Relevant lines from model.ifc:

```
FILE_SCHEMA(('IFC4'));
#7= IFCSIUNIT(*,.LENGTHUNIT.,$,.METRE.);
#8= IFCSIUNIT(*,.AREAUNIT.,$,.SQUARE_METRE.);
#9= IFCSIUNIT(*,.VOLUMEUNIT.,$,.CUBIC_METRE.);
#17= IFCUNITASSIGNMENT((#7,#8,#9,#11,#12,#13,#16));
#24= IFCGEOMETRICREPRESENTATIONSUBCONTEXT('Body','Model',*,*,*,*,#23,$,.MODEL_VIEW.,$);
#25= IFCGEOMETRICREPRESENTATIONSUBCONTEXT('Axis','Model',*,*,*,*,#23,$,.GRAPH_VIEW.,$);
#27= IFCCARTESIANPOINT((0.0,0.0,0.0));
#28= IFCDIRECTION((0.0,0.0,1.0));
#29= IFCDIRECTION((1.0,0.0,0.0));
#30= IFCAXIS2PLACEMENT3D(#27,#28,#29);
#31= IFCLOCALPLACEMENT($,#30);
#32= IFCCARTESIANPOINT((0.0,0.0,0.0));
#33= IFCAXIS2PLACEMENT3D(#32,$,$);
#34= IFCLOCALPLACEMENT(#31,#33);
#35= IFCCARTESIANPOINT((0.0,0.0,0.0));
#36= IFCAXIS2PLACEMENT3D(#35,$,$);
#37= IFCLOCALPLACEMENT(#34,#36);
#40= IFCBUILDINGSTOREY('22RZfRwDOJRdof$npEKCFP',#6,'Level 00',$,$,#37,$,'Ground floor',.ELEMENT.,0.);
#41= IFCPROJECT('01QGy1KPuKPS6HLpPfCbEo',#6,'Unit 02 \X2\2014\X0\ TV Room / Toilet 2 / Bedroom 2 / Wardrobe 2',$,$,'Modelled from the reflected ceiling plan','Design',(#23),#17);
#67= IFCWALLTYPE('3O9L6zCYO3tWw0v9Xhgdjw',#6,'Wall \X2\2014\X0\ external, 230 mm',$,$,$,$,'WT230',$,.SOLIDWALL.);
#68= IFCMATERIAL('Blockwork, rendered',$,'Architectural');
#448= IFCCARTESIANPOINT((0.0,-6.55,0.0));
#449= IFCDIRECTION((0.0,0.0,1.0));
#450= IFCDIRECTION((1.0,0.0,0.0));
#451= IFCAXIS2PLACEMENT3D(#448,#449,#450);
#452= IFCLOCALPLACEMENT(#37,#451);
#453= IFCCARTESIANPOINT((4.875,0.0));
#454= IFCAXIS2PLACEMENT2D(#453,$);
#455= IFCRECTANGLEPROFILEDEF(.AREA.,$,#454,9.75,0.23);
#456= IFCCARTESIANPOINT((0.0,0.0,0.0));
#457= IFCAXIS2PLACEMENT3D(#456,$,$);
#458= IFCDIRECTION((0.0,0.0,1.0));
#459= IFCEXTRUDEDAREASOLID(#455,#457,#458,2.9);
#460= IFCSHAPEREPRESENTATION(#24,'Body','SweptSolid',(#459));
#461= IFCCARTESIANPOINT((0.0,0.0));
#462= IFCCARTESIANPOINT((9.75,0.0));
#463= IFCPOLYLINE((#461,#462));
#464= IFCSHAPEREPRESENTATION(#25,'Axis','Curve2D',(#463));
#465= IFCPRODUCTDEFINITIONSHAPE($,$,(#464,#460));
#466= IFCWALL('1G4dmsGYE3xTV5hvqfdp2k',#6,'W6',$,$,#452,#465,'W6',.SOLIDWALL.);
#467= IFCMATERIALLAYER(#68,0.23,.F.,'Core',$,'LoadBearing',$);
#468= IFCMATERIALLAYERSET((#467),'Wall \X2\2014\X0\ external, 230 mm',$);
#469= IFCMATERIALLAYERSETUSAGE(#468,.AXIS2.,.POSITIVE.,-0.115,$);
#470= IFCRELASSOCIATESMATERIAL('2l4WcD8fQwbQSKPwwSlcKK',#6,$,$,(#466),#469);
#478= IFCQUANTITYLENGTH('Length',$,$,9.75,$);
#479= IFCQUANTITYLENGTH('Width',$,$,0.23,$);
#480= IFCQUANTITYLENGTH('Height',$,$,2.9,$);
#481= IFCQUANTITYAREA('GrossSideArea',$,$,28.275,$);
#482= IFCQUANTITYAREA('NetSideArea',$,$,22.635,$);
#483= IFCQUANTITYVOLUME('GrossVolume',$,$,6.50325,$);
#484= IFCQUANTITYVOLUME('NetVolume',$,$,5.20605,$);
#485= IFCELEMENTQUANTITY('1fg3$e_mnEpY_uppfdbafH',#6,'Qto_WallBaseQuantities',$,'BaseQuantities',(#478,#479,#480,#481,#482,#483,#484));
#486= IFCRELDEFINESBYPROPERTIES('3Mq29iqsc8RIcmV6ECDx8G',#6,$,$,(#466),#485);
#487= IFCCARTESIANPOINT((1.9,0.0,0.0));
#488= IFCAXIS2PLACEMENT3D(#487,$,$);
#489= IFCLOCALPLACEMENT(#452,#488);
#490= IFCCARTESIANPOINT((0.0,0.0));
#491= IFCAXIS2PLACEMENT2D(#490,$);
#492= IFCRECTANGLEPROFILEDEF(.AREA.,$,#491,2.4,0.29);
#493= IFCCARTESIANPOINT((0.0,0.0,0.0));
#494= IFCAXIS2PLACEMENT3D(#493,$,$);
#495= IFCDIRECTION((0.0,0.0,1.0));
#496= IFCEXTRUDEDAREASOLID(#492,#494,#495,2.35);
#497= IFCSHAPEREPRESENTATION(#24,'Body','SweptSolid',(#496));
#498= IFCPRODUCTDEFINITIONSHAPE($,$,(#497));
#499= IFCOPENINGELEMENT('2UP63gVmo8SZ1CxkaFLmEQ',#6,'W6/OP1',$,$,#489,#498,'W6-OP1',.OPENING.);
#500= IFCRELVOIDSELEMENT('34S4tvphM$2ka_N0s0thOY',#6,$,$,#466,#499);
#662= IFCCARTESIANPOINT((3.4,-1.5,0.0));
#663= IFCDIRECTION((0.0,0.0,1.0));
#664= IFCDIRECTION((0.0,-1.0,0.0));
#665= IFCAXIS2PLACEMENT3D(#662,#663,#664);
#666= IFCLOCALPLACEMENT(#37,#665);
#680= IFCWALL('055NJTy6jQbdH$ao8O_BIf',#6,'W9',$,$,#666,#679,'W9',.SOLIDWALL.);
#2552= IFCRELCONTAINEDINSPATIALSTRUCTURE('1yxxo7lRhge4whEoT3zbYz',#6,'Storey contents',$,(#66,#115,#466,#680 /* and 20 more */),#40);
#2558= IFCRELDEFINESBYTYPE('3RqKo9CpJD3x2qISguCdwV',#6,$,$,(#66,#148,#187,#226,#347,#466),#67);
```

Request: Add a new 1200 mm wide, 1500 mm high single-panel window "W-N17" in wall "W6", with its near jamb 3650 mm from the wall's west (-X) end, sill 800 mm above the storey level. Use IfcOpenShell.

```python
import numpy as np
import ifcopenshell
import ifcopenshell.api.feature
import ifcopenshell.api.geometry
import ifcopenshell.api.pset
import ifcopenshell.api.root
import ifcopenshell.api.spatial
import ifcopenshell.geom
import ifcopenshell.util.element
import ifcopenshell.util.placement
import ifcopenshell.util.representation
import ifcopenshell.util.shape
import ifcopenshell.util.unit

model = ifcopenshell.open("model.ifc")
unit_scale = ifcopenshell.util.unit.calculate_unit_scale(model)
area_scale = ifcopenshell.util.unit.calculate_unit_scale(model, "AREAUNIT")
volume_scale = ifcopenshell.util.unit.calculate_unit_scale(model, "VOLUMEUNIT")
settings = ifcopenshell.geom.settings()


def volume(element):
    """Net volume in cubic metres, openings subtracted."""
    shape = ifcopenshell.geom.create_shape(settings, element)
    return ifcopenshell.util.shape.get_volume(shape.geometry)


wall = model.by_id(466)
storey = ifcopenshell.util.element.get_container(wall, ifc_class="IfcBuildingStorey")
context = ifcopenshell.util.representation.get_context(model, "Model", "Body", "MODEL_VIEW")
before = volume(wall)

width, height, from_end, sill = 1.2, 1.5, 3.65, 0.8  # metres

# The wall runs along its own X axis, and the end named is its -X end.
wall_shape = ifcopenshell.geom.create_shape(settings, wall)
x, y, z = ifcopenshell.util.shape.get_vertices(wall_shape.geometry).T
start = x.min() + from_end
face, thickness = float(y.min()), float(y.max() - y.min())
wall_matrix = ifcopenshell.util.placement.get_local_placement(wall.ObjectPlacement)
level = ifcopenshell.util.placement.get_local_placement(storey.ObjectPlacement)[2, 3]


def in_wall(x, y):
    """Placement at x, y metres in the wall's axes, at sill height."""
    matrix = wall_matrix.copy()
    matrix[:, 3] = wall_matrix @ np.array([x / unit_scale, y / unit_scale, 0.0, 1.0])
    matrix[2, 3] = level + sill / unit_scale
    return matrix


# Opening: a box that overshoots both wall faces by 50 mm.
opening = ifcopenshell.api.root.create_entity(model, ifc_class="IfcOpeningElement", predefined_type="OPENING")
box = ifcopenshell.api.geometry.add_wall_representation(
    model, context=context, length=width, height=height, thickness=thickness + 0.1
)
ifcopenshell.api.geometry.assign_representation(model, product=opening, representation=box)
ifcopenshell.api.geometry.edit_object_placement(model, product=opening, matrix=in_wall(start, face - 0.05), is_si=False)
ifcopenshell.api.feature.add_feature(model, feature=opening, element=wall)

window = ifcopenshell.api.root.create_entity(model, ifc_class="IfcWindow", name="W-N17", predefined_type="WINDOW")
window.OverallWidth, window.OverallHeight = width / unit_scale, height / unit_scale
window.PartitioningType = "SINGLE_PANEL"
body = ifcopenshell.api.geometry.add_window_representation(
    model,
    context=context,
    overall_width=window.OverallWidth,
    overall_height=window.OverallHeight,
    partition_type="SINGLE_PANEL",
)
ifcopenshell.api.geometry.assign_representation(model, product=window, representation=body)
ifcopenshell.api.spatial.assign_container(model, products=[window], relating_structure=storey)
ifcopenshell.api.feature.add_filling(model, opening=opening, element=window)

# Centre the window in the wall's thickness.
ifcopenshell.api.geometry.edit_object_placement(model, product=window, matrix=in_wall(start, face), is_si=False)
window_shape = ifcopenshell.geom.create_shape(settings, window)
depth = ifcopenshell.util.shape.get_vertices(window_shape.geometry)[:, 1]
offset = face + thickness / 2 - (depth.min() + depth.max()) / 2
ifcopenshell.api.geometry.edit_object_placement(model, product=window, matrix=in_wall(start, offset), is_si=False)

after = volume(wall)

# Update the wall's stored quantities.
qto = model.by_id(ifcopenshell.util.element.get_pset(wall, "Qto_WallBaseQuantities", should_inherit=False)["id"])
ifcopenshell.api.pset.edit_qto(model, qto=qto, properties={
    "NetSideArea": after / thickness / area_scale,
    "NetVolume": after / volume_scale,
})

print(f"wall volume {before:.3f} -> {after:.3f} m3")

model.write("model_v2.ifc")
```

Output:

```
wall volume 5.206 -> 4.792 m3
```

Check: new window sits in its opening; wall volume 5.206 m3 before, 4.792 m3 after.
